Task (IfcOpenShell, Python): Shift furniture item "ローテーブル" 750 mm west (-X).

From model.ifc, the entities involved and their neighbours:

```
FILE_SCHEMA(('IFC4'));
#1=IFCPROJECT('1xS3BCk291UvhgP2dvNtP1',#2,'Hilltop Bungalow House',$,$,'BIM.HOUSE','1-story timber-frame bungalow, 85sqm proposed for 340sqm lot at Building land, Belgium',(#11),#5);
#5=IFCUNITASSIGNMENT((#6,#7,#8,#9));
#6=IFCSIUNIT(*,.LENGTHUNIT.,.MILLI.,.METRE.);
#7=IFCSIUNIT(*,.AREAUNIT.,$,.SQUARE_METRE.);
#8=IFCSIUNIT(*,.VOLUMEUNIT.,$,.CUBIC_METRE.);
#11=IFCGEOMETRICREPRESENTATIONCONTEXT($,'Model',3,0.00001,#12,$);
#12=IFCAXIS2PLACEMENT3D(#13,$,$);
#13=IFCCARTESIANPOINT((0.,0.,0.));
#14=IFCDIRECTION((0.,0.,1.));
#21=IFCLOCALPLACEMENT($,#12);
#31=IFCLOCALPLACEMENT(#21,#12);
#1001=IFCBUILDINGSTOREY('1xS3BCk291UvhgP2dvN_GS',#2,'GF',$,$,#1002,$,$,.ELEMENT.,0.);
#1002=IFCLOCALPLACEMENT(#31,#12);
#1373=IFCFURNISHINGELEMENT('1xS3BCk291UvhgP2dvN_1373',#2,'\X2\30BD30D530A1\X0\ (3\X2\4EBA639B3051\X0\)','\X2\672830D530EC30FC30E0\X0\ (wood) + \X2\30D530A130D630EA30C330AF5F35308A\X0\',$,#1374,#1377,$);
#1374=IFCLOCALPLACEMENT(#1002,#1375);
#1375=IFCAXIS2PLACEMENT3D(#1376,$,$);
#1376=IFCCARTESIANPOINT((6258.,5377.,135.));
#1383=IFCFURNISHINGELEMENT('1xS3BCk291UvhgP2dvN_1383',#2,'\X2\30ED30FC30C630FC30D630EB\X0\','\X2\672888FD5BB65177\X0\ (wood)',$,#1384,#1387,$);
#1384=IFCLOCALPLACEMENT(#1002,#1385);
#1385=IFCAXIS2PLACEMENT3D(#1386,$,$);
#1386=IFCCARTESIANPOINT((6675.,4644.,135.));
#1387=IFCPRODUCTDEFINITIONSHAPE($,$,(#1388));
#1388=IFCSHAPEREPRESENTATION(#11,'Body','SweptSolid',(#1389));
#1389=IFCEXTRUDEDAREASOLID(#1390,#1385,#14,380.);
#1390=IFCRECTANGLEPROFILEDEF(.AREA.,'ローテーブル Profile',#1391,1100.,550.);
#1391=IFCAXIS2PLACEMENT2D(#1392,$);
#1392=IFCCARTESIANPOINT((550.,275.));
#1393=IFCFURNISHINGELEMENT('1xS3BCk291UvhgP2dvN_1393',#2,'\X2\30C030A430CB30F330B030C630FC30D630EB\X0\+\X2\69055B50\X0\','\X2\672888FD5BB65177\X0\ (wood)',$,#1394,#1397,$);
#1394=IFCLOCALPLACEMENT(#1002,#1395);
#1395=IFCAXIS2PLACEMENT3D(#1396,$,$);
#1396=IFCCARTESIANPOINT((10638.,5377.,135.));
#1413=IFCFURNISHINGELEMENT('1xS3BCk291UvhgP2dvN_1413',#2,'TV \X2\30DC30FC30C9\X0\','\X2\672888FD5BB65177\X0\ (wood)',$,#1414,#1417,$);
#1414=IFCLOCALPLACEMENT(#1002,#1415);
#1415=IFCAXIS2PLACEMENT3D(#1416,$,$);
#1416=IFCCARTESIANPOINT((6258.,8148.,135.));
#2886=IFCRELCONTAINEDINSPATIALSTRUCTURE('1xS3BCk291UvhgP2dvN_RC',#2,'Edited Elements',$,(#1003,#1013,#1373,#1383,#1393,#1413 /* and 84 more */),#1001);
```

```python
import ifcopenshell
import ifcopenshell.api.geometry
import ifcopenshell.util.placement
import ifcopenshell.util.unit

model = ifcopenshell.open("model.ifc")
unit_scale = ifcopenshell.util.unit.calculate_unit_scale(model)

item = model.by_id(1383)
matrix = ifcopenshell.util.placement.get_local_placement(item.ObjectPlacement)
matrix[0, 3] -= 0.75 / unit_scale
ifcopenshell.api.geometry.edit_object_placement(model, product=item, matrix=matrix, is_si=False)

print(ifcopenshell.util.placement.get_local_placement(item.ObjectPlacement).round(3) + 0.0)

model.write("model_v2.ifc")
```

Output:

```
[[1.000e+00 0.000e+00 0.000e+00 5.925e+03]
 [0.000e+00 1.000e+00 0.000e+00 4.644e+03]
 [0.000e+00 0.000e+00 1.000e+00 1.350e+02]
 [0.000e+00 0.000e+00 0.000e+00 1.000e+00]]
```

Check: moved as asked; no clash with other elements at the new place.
